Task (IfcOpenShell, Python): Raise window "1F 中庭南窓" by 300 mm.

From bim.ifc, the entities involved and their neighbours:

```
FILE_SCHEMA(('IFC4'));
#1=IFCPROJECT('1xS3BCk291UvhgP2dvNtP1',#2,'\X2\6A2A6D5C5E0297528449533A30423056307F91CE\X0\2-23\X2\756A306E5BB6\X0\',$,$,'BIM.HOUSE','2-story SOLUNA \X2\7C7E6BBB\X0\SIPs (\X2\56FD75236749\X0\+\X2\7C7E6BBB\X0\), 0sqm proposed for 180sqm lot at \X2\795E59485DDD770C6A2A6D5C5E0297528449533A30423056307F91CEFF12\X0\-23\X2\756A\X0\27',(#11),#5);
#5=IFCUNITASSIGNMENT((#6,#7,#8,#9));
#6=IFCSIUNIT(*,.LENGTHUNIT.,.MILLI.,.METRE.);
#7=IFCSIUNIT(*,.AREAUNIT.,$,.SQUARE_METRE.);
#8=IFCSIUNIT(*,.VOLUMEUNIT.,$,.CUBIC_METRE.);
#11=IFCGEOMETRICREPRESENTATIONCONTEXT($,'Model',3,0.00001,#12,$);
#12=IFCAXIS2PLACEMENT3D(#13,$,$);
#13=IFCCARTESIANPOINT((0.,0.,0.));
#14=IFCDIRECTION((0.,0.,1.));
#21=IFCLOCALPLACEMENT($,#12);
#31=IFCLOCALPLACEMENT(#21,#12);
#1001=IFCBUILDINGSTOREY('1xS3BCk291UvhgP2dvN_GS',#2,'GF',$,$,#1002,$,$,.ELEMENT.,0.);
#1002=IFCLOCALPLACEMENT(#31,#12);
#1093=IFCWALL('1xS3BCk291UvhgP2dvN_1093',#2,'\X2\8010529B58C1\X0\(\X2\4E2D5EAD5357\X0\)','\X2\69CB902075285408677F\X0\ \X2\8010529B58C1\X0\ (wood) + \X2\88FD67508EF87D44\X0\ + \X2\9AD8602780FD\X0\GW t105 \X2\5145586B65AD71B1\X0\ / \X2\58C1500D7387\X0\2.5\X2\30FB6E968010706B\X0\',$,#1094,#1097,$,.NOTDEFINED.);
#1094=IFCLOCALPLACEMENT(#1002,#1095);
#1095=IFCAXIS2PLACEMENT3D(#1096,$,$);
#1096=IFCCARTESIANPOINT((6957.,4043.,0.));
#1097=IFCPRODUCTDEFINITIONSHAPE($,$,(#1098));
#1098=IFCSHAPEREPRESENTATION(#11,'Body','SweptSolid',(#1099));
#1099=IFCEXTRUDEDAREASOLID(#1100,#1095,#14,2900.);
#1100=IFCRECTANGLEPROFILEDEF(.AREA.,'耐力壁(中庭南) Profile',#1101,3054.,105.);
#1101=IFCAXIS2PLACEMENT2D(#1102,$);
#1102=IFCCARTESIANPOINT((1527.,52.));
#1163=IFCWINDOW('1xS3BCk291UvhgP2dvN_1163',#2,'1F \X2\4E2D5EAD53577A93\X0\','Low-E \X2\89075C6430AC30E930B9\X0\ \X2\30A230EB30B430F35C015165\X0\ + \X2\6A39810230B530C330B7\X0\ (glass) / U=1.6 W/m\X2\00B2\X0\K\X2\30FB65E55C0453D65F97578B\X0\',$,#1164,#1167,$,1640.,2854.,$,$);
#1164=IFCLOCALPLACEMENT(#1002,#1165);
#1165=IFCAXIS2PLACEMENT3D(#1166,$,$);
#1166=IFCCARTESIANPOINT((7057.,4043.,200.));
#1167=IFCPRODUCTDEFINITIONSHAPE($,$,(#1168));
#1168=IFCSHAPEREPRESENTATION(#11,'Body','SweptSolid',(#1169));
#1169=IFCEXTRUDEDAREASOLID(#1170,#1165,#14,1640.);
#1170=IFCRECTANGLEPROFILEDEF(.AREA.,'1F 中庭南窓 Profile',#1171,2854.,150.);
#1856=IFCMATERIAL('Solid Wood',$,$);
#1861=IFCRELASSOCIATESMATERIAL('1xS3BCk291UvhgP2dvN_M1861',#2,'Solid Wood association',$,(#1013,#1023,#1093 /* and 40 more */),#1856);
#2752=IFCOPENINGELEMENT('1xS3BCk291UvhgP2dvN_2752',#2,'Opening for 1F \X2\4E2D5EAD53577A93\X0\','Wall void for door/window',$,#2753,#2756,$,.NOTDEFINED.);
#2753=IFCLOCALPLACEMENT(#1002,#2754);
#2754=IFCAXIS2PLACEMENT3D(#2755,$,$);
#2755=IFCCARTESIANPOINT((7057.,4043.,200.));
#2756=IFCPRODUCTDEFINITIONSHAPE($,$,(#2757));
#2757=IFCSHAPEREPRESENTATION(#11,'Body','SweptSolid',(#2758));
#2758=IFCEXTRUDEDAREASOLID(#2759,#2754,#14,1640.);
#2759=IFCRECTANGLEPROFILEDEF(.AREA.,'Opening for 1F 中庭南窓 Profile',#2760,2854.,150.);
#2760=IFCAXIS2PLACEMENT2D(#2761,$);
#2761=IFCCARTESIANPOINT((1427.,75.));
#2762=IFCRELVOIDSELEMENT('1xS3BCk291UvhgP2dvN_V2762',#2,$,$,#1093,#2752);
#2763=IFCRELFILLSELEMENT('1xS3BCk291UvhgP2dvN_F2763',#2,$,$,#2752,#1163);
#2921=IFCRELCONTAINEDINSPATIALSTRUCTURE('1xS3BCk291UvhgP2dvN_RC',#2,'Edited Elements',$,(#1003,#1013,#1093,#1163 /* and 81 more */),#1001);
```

```python
import numpy as np
import ifcopenshell
import ifcopenshell.api.geometry
import ifcopenshell.util.placement
import ifcopenshell.util.unit

model = ifcopenshell.open("bim.ifc")
unit_scale = ifcopenshell.util.unit.calculate_unit_scale(model)

window = model.by_guid("1xS3BCk291UvhgP2dvN_1163")
opening = window.FillsVoids[0].RelatingOpeningElement
dz = 0.3 / unit_scale

shift = np.array([0.0, 0.0, dz])
# The window is not placed relative to its opening, so move both.
for product in (opening, window):
    matrix = ifcopenshell.util.placement.get_local_placement(product.ObjectPlacement)
    matrix[:3, 3] += shift
    ifcopenshell.api.geometry.edit_object_placement(model, product=product, matrix=matrix, is_si=False)

print(f"moved by {dz * unit_scale:+.3f} m")

model.write("bim_edited.ifc")
```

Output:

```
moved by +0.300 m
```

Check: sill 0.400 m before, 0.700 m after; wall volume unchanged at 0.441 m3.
